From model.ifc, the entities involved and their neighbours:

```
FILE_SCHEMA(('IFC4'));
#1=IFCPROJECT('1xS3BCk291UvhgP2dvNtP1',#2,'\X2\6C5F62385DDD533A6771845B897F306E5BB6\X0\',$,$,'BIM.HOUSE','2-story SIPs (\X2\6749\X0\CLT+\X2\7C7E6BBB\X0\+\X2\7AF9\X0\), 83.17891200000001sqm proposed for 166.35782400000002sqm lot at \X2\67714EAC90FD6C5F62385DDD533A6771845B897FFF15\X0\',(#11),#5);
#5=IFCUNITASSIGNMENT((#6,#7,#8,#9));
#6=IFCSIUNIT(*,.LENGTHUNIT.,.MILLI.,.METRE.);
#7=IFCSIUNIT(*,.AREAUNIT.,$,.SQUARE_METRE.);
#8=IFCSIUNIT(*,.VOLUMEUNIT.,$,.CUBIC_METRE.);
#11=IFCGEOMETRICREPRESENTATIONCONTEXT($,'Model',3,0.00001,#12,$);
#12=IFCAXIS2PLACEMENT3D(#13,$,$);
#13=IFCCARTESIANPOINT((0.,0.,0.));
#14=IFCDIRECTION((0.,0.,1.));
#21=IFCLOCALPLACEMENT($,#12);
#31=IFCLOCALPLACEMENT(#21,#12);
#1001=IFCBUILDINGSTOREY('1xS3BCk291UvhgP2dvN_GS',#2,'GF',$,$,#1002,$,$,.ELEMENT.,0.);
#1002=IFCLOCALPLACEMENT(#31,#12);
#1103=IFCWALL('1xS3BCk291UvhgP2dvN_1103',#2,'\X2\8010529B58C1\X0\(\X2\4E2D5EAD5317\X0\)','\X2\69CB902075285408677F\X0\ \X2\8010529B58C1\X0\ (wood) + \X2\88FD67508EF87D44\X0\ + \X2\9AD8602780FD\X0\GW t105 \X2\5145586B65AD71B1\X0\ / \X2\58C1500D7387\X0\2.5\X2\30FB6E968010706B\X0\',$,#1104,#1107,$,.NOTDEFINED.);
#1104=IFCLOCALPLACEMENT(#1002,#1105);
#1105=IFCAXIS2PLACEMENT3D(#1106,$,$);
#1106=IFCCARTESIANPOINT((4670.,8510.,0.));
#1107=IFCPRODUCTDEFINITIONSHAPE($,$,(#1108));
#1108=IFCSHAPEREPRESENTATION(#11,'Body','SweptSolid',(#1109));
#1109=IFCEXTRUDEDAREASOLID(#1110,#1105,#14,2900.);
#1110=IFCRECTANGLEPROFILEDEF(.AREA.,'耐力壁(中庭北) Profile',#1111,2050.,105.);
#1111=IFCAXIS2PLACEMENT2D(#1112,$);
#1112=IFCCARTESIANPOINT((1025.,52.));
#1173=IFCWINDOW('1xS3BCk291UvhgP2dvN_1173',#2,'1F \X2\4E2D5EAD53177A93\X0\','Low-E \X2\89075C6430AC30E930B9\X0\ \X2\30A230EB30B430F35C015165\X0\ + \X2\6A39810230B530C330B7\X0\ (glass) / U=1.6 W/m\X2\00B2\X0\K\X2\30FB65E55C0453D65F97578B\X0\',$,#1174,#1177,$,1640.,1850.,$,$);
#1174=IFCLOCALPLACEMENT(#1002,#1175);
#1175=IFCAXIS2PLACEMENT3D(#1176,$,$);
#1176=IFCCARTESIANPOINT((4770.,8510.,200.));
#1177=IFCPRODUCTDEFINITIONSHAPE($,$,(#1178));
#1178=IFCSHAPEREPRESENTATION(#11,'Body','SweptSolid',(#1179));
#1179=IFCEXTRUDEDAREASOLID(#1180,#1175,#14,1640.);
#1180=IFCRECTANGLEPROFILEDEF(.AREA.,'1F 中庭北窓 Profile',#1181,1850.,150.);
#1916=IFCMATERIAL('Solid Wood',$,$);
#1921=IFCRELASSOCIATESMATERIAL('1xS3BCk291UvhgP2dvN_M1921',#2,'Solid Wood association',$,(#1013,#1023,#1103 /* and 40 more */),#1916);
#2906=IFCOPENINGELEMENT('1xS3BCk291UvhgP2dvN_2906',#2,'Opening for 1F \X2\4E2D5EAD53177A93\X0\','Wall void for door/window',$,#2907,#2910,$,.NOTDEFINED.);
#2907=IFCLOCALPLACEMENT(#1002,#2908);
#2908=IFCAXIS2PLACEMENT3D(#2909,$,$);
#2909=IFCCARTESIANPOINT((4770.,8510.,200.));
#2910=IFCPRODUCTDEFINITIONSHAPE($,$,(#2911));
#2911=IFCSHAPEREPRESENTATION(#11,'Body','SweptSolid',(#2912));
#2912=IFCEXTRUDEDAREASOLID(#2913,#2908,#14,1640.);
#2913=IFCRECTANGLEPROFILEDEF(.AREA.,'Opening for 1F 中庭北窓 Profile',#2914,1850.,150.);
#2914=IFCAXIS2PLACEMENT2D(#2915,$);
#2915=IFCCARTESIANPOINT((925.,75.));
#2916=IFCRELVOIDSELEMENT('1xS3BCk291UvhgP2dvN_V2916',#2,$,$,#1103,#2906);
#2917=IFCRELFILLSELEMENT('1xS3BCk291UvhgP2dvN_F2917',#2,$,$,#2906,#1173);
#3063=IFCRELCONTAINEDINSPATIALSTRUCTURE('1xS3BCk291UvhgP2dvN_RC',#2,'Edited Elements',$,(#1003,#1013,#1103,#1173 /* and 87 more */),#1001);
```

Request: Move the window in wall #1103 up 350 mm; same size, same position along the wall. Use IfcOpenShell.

```python
import numpy as np
import ifcopenshell
import ifcopenshell.api.geometry
import ifcopenshell.util.placement
import ifcopenshell.util.unit

model = ifcopenshell.open("model.ifc")
unit_scale = ifcopenshell.util.unit.calculate_unit_scale(model)

window = model.by_guid("1xS3BCk291UvhgP2dvN_1173")
opening = window.FillsVoids[0].RelatingOpeningElement
dz = 0.35 / unit_scale

shift = np.array([0.0, 0.0, dz])
# The window is not placed relative to its opening, so move both.
for product in (opening, window):
    matrix = ifcopenshell.util.placement.get_local_placement(product.ObjectPlacement)
    matrix[:3, 3] += shift
    ifcopenshell.api.geometry.edit_object_placement(model, product=product, matrix=matrix, is_si=False)

print(f"moved by {dz * unit_scale:+.3f} m")

model.write("model_v2.ifc")
```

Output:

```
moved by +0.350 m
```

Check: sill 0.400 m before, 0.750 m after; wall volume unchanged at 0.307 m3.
